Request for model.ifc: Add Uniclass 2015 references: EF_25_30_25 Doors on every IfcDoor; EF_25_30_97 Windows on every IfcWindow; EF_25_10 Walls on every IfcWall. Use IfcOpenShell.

First a look at what the model holds.

```python
import ifcopenshell

model = ifcopenshell.open("model.ifc")
print(model.schema)
print("classifications:", [c.Name for c in model.by_type("IfcClassification")])
for ifc_class in ("IfcDoor", "IfcRoof", "IfcStair", "IfcWall", "IfcWindow"):
    print(ifc_class, len(model.by_type(ifc_class)))
```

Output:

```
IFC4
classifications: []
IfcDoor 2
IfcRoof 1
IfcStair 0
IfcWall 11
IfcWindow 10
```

```python
import ifcopenshell
import ifcopenshell.api.classification

model = ifcopenshell.open("model.ifc")

system = ifcopenshell.api.classification.add_classification(model, classification="Uniclass 2015")

codes = {
    "IfcDoor": ("EF_25_30_25", "Doors"),
    "IfcWindow": ("EF_25_30_97", "Windows"),
    "IfcWall": ("EF_25_10", "Walls"),
}
for ifc_class, (code, name) in codes.items():
    products = model.by_type(ifc_class)
    ifcopenshell.api.classification.add_reference(
        model, products=products, classification=system, identification=code, name=name
    )
    print(code, len(products))

model.write("model_updated.ifc")
```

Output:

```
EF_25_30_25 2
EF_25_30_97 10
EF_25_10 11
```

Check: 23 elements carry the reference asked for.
